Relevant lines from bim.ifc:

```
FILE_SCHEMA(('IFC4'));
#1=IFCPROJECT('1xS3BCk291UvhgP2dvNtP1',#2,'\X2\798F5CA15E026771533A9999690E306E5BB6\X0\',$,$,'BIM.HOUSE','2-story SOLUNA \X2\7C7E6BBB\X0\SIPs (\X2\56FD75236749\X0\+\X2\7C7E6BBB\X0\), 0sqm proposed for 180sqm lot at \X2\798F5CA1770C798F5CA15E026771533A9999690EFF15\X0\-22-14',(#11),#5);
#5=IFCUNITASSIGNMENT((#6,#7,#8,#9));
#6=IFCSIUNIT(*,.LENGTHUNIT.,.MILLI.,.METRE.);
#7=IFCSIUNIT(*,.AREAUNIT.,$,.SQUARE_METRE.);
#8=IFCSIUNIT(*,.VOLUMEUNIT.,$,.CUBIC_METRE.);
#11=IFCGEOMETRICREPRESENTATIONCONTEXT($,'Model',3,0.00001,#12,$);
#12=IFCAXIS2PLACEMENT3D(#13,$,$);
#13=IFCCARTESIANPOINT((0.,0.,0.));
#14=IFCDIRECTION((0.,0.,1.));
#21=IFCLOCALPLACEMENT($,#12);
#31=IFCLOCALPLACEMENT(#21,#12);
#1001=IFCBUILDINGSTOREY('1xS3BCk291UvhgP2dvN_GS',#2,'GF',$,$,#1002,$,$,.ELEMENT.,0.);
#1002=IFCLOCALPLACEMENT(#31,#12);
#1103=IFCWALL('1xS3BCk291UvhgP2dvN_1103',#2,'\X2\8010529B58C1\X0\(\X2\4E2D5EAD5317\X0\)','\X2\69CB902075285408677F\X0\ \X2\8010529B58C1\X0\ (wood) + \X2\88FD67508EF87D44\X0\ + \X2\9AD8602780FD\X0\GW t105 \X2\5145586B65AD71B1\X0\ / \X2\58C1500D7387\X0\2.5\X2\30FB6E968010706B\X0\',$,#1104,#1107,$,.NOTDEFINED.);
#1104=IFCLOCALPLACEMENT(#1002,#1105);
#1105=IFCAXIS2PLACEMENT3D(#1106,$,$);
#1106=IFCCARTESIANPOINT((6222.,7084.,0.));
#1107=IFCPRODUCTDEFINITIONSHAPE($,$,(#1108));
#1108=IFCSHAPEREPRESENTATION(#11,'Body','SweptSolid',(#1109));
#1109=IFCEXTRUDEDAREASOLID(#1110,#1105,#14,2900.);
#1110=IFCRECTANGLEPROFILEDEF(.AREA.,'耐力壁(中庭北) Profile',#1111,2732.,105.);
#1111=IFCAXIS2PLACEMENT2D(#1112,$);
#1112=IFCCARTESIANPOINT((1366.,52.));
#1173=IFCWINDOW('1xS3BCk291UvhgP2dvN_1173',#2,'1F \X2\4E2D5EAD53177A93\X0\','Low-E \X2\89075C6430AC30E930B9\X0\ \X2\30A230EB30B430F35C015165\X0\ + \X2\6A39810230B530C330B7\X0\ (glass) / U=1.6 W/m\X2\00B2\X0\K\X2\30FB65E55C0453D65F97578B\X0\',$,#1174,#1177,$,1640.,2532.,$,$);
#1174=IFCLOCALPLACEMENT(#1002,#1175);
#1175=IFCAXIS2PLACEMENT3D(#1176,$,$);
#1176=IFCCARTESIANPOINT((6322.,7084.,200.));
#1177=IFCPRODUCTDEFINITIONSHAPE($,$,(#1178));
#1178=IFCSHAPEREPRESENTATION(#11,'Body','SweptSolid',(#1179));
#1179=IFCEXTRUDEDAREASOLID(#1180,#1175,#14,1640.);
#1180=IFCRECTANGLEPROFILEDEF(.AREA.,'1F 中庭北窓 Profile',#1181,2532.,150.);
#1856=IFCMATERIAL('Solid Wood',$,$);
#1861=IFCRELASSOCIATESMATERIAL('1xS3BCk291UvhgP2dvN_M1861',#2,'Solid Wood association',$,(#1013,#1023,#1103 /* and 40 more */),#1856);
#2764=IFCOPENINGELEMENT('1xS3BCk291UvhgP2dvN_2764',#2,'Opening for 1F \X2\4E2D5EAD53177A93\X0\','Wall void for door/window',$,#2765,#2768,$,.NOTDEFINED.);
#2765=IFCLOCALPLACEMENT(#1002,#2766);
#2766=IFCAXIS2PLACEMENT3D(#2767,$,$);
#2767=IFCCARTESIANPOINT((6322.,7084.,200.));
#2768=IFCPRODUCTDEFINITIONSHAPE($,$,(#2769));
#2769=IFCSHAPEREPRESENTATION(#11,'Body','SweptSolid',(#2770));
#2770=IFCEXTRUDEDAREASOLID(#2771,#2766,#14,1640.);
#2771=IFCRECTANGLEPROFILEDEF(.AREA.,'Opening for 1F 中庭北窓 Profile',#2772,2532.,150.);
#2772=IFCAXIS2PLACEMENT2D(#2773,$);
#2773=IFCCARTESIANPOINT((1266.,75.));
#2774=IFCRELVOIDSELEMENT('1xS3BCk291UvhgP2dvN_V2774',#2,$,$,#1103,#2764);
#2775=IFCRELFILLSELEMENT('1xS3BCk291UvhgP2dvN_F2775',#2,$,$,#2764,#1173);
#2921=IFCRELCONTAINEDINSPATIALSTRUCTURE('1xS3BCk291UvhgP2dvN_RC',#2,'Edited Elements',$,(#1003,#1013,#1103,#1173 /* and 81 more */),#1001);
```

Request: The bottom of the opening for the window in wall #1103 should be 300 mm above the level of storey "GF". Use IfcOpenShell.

```python
import numpy as np
import ifcopenshell
import ifcopenshell.api.geometry
import ifcopenshell.geom
import ifcopenshell.util.element
import ifcopenshell.util.placement
import ifcopenshell.util.shape
import ifcopenshell.util.unit

model = ifcopenshell.open("bim.ifc")
unit_scale = ifcopenshell.util.unit.calculate_unit_scale(model)

window = model.by_id(1173)
opening = window.FillsVoids[0].RelatingOpeningElement
storey = ifcopenshell.util.element.get_container(window, ifc_class="IfcBuildingStorey")
level = ifcopenshell.util.placement.get_local_placement(storey.ObjectPlacement)[2, 3]

# The opening's origin need not be at the sill, so measure its lowest point.
shape = ifcopenshell.geom.create_shape(ifcopenshell.geom.settings(), opening)
bottom = ifcopenshell.util.shape.get_shape_bottom_elevation(shape, shape.geometry) / unit_scale
dz = level + 0.3 / unit_scale - bottom

shift = np.array([0.0, 0.0, dz])
# The window is not placed relative to its opening, so move both.
for product in (opening, window):
    matrix = ifcopenshell.util.placement.get_local_placement(product.ObjectPlacement)
    matrix[:3, 3] += shift
    ifcopenshell.api.geometry.edit_object_placement(model, product=product, matrix=matrix, is_si=False)

print(f"moved by {dz * unit_scale:+.3f} m")

model.write("bim_rev.ifc")
```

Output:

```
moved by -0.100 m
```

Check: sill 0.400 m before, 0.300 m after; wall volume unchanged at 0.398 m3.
